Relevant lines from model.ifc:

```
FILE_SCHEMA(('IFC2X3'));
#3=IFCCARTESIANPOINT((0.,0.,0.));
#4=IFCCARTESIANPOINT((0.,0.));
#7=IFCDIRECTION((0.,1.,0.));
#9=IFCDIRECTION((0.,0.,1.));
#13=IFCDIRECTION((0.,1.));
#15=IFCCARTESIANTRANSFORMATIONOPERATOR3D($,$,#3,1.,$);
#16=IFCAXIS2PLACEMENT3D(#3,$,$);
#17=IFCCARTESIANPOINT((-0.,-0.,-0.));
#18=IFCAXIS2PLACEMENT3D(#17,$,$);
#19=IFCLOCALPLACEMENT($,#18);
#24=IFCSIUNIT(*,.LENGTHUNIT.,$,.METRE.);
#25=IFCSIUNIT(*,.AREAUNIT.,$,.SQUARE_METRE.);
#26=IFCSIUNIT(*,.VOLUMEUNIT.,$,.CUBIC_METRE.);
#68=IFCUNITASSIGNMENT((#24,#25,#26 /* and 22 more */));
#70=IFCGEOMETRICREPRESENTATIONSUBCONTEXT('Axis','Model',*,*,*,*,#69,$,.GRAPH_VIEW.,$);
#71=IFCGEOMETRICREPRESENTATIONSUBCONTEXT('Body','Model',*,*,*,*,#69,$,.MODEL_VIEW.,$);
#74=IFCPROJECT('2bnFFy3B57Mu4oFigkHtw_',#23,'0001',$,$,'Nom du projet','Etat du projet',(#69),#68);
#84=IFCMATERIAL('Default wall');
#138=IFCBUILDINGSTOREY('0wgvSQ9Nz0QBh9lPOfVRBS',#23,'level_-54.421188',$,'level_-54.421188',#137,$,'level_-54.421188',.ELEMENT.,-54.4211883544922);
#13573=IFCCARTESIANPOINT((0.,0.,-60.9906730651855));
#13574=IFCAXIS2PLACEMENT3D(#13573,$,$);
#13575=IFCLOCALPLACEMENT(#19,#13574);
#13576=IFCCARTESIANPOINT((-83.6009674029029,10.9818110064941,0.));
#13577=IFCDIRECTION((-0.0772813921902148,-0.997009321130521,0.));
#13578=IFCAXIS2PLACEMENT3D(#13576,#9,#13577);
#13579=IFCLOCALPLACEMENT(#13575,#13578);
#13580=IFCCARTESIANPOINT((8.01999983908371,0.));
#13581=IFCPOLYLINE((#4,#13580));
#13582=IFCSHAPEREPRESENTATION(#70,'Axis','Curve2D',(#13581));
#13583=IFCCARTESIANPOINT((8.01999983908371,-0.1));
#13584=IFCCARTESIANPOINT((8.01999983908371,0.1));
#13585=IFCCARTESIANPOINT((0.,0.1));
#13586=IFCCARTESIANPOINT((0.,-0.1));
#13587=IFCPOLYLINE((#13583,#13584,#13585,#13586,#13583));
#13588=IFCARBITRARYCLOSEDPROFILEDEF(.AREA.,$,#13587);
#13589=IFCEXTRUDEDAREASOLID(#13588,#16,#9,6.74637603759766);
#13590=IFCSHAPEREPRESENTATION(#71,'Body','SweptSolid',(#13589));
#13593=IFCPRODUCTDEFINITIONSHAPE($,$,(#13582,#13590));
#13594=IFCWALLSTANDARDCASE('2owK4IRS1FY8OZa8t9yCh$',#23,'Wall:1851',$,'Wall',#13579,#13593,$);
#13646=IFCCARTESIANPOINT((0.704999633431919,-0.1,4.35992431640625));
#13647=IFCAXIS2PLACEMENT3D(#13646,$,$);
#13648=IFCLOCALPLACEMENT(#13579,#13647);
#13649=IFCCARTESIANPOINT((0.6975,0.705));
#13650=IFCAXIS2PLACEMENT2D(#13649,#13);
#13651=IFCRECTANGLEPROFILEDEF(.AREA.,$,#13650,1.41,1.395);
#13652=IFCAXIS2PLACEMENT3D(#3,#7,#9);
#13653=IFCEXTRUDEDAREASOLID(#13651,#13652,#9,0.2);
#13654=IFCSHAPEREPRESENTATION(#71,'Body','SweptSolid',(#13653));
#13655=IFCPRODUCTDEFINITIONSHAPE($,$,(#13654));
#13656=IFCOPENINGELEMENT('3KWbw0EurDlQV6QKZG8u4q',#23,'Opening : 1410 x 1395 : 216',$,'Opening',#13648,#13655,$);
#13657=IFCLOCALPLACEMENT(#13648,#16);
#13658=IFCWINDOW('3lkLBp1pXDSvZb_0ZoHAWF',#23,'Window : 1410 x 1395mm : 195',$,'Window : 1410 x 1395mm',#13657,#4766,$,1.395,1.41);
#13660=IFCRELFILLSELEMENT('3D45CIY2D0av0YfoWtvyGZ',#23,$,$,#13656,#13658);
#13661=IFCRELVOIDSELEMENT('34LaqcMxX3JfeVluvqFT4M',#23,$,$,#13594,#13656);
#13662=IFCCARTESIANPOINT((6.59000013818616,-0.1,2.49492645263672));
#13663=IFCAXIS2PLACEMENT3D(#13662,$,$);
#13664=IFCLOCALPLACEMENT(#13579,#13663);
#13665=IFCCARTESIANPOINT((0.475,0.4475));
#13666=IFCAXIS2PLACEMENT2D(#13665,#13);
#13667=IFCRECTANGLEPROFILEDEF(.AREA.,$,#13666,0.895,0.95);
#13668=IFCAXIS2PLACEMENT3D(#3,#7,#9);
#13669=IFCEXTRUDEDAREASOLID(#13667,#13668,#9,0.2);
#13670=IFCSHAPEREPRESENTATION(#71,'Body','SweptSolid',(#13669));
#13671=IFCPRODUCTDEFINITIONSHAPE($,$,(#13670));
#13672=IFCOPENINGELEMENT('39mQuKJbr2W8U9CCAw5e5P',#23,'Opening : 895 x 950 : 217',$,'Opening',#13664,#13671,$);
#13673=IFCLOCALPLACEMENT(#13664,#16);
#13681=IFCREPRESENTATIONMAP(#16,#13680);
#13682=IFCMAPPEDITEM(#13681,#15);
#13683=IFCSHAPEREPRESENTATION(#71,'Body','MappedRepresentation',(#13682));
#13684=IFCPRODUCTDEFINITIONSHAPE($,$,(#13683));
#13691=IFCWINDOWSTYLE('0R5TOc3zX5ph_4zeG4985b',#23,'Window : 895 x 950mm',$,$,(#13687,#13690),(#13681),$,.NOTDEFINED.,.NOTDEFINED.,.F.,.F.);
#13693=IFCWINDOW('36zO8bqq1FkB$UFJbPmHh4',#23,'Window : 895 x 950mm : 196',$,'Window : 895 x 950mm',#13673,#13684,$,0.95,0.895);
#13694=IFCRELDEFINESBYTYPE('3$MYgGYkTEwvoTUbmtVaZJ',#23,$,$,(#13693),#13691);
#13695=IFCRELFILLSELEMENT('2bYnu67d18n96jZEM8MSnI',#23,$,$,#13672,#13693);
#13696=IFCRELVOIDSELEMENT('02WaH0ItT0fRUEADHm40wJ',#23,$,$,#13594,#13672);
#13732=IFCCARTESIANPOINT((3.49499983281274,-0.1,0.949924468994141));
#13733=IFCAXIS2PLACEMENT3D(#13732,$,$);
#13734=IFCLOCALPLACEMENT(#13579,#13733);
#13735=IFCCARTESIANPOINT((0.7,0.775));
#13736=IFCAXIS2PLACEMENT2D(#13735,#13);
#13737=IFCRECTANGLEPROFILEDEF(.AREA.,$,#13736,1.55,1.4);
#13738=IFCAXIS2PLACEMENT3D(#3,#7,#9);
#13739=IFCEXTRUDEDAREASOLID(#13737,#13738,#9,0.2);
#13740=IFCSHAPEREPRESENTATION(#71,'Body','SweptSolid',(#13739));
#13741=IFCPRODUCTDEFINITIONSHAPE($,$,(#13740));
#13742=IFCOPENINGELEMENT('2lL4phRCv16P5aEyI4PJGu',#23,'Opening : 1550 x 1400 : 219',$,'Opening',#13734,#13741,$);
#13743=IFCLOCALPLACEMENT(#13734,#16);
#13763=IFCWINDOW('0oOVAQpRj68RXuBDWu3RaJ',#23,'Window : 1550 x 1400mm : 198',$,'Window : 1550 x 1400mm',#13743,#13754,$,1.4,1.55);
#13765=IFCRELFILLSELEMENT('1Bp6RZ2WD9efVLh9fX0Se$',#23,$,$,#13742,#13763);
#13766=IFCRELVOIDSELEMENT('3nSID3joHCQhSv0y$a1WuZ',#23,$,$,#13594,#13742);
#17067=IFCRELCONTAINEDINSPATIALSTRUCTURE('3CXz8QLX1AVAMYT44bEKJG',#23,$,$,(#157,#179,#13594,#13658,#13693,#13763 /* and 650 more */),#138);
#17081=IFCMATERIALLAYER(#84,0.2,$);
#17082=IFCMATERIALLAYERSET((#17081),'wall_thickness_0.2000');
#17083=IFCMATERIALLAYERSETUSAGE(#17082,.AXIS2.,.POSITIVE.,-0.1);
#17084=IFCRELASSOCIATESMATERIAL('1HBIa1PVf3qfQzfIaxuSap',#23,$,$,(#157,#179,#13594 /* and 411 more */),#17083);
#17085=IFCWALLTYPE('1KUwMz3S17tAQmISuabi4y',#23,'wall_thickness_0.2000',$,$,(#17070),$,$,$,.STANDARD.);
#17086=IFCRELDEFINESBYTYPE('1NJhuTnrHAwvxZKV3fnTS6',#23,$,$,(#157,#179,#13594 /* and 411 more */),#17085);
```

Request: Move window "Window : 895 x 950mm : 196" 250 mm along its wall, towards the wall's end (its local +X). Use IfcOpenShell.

```python
import ifcopenshell
import ifcopenshell.api.geometry
import ifcopenshell.util.placement

model = ifcopenshell.open("model.ifc")

window = model.by_guid("36zO8bqq1FkB$UFJbPmHh4")
opening = window.FillsVoids[0].RelatingOpeningElement
wall = opening.VoidsElements[0].RelatingBuildingElement

wall_matrix = ifcopenshell.util.placement.get_local_placement(wall.ObjectPlacement)
shift = wall_matrix[:3, 0] * 0.25
before = ifcopenshell.util.placement.get_local_placement(window.ObjectPlacement)[:3, 3].copy()

# The window is placed relative to its opening, so it follows when the opening moves.
matrix = ifcopenshell.util.placement.get_local_placement(opening.ObjectPlacement)
matrix[:3, 3] += shift
ifcopenshell.api.geometry.edit_object_placement(
    model, product=opening, matrix=matrix, is_si=False, should_transform_children=True
)

after = ifcopenshell.util.placement.get_local_placement(window.ObjectPlacement)[:3, 3]
print("window moved by", (after - before).round(3) + 0.0)

model.write("model_edited.ifc")
```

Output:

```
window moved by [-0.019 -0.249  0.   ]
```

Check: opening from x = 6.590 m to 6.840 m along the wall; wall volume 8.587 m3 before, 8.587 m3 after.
